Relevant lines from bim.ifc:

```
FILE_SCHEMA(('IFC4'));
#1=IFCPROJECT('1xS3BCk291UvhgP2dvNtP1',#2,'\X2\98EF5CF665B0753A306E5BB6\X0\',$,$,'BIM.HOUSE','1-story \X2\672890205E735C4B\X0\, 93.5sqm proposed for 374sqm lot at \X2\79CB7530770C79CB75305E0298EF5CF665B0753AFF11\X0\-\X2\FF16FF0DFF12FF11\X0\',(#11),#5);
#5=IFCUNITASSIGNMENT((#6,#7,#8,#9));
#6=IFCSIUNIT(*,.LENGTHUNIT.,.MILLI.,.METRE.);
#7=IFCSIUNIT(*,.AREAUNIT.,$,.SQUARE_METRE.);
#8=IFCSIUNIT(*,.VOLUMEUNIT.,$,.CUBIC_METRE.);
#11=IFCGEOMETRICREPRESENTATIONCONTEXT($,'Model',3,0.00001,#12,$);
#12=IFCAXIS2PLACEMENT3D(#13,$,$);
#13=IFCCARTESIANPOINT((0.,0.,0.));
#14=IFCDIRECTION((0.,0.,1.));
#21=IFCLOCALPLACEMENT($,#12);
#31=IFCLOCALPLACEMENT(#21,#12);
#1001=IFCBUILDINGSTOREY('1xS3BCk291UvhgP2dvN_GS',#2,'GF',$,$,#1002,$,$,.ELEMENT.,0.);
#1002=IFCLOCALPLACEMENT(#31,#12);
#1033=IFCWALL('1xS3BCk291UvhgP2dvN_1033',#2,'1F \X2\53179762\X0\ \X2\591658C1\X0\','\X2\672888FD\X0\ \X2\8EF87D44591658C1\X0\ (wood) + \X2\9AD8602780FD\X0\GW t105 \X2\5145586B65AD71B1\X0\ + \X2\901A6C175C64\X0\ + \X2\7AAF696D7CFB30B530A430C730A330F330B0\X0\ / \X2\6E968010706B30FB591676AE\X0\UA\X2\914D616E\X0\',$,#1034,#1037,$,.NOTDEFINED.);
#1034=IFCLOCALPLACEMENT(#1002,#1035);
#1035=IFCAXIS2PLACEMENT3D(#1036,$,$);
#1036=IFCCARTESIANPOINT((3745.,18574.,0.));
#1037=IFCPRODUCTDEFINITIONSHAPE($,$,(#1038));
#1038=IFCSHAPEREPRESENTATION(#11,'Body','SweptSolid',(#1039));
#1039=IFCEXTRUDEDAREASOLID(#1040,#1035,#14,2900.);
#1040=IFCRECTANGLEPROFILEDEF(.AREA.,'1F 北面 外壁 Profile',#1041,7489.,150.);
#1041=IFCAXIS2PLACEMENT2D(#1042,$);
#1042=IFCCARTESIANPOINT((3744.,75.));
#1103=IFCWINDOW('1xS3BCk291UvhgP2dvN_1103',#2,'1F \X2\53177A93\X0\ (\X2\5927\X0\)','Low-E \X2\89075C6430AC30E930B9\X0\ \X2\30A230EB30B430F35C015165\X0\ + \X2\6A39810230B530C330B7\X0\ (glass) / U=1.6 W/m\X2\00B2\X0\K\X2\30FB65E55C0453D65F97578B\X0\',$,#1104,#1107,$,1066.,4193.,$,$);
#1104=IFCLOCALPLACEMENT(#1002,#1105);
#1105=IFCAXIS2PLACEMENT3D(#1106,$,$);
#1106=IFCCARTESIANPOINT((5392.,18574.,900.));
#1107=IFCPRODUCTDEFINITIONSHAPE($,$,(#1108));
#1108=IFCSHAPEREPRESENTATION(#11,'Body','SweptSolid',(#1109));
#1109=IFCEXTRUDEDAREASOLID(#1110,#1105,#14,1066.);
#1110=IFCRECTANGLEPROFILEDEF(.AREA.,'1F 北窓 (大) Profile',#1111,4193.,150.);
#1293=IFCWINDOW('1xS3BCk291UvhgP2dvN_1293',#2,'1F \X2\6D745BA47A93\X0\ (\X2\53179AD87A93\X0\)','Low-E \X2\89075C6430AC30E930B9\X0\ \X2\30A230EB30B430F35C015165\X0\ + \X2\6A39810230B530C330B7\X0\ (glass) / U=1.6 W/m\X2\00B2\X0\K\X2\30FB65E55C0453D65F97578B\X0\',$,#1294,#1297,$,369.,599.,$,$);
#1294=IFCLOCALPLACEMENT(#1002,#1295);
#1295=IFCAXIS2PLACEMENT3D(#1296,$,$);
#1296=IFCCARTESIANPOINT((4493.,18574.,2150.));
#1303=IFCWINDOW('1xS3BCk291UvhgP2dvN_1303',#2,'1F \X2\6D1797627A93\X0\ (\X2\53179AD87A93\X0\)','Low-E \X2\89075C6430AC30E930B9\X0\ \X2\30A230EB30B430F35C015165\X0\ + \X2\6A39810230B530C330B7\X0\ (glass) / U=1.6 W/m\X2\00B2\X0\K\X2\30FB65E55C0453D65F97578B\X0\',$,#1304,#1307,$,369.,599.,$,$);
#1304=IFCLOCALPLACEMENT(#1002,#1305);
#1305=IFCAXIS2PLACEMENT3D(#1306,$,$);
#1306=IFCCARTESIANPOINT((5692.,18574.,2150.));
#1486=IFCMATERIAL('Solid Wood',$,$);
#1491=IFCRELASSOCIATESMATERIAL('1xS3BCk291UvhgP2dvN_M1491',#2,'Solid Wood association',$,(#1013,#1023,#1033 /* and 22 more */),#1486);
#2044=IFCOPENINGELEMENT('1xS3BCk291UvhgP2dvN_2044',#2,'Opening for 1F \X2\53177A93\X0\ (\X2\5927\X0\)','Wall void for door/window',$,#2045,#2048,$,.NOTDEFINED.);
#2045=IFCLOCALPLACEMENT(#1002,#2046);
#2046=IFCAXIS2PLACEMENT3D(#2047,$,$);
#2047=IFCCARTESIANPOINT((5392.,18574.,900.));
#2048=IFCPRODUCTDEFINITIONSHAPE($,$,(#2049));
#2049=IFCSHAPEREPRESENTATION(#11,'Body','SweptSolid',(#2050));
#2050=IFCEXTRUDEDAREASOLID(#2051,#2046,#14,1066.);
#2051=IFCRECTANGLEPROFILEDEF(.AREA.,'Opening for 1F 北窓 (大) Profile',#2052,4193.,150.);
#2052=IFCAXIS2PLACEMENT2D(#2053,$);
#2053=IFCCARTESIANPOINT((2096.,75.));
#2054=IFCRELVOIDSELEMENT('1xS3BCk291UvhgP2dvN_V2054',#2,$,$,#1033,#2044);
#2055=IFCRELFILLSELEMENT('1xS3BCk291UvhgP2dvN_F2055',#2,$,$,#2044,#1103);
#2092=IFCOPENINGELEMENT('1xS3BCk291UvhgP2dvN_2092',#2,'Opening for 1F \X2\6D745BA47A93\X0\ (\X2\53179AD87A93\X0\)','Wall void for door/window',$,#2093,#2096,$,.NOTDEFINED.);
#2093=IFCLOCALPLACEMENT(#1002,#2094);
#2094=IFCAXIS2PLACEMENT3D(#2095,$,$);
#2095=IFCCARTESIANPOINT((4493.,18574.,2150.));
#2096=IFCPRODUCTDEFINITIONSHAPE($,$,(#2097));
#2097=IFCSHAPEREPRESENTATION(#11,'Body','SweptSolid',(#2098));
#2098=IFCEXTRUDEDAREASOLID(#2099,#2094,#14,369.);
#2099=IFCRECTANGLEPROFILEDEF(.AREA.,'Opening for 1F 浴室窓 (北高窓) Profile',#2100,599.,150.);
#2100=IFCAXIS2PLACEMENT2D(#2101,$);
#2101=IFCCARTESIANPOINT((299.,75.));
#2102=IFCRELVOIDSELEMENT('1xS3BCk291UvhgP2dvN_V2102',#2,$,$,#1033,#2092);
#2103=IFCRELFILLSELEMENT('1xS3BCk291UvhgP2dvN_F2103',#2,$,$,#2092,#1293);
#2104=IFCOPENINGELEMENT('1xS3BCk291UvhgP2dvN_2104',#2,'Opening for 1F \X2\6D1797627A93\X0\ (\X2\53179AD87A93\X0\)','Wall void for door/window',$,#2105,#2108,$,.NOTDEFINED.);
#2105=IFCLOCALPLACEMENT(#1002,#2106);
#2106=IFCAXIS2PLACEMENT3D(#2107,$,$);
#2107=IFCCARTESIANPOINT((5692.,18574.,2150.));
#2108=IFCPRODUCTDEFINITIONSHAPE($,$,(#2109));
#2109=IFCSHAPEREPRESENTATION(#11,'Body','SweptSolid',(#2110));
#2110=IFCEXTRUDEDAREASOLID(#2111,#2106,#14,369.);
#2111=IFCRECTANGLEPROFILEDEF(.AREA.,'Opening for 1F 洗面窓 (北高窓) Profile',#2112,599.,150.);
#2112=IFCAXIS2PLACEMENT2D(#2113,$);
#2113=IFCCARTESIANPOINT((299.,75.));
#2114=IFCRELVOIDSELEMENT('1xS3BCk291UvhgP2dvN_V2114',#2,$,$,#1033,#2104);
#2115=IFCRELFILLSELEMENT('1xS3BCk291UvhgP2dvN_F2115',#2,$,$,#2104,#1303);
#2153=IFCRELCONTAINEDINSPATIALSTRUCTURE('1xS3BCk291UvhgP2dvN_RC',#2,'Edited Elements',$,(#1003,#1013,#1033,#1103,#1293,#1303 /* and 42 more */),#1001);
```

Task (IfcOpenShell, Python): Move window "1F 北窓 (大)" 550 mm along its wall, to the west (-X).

```python
import ifcopenshell
import ifcopenshell.api.geometry
import ifcopenshell.util.placement
import ifcopenshell.util.unit

model = ifcopenshell.open("bim.ifc")
unit_scale = ifcopenshell.util.unit.calculate_unit_scale(model)

window = model.by_guid("1xS3BCk291UvhgP2dvN_1103")
opening = window.FillsVoids[0].RelatingOpeningElement
wall = opening.VoidsElements[0].RelatingBuildingElement

wall_matrix = ifcopenshell.util.placement.get_local_placement(wall.ObjectPlacement)
shift = wall_matrix[:3, 0] * -0.55 / unit_scale
before = ifcopenshell.util.placement.get_local_placement(window.ObjectPlacement)[:3, 3].copy()

# The window is not placed relative to its opening, so move both.
for product in (opening, window):
    matrix = ifcopenshell.util.placement.get_local_placement(product.ObjectPlacement)
    matrix[:3, 3] += shift
    ifcopenshell.api.geometry.edit_object_placement(model, product=product, matrix=matrix, is_si=False)

after = ifcopenshell.util.placement.get_local_placement(window.ObjectPlacement)[:3, 3]
print("window moved by", (after - before).round(3) + 0.0)

model.write("bim_edited.ifc")
```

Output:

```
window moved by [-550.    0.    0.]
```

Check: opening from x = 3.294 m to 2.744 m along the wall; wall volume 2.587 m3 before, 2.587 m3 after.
